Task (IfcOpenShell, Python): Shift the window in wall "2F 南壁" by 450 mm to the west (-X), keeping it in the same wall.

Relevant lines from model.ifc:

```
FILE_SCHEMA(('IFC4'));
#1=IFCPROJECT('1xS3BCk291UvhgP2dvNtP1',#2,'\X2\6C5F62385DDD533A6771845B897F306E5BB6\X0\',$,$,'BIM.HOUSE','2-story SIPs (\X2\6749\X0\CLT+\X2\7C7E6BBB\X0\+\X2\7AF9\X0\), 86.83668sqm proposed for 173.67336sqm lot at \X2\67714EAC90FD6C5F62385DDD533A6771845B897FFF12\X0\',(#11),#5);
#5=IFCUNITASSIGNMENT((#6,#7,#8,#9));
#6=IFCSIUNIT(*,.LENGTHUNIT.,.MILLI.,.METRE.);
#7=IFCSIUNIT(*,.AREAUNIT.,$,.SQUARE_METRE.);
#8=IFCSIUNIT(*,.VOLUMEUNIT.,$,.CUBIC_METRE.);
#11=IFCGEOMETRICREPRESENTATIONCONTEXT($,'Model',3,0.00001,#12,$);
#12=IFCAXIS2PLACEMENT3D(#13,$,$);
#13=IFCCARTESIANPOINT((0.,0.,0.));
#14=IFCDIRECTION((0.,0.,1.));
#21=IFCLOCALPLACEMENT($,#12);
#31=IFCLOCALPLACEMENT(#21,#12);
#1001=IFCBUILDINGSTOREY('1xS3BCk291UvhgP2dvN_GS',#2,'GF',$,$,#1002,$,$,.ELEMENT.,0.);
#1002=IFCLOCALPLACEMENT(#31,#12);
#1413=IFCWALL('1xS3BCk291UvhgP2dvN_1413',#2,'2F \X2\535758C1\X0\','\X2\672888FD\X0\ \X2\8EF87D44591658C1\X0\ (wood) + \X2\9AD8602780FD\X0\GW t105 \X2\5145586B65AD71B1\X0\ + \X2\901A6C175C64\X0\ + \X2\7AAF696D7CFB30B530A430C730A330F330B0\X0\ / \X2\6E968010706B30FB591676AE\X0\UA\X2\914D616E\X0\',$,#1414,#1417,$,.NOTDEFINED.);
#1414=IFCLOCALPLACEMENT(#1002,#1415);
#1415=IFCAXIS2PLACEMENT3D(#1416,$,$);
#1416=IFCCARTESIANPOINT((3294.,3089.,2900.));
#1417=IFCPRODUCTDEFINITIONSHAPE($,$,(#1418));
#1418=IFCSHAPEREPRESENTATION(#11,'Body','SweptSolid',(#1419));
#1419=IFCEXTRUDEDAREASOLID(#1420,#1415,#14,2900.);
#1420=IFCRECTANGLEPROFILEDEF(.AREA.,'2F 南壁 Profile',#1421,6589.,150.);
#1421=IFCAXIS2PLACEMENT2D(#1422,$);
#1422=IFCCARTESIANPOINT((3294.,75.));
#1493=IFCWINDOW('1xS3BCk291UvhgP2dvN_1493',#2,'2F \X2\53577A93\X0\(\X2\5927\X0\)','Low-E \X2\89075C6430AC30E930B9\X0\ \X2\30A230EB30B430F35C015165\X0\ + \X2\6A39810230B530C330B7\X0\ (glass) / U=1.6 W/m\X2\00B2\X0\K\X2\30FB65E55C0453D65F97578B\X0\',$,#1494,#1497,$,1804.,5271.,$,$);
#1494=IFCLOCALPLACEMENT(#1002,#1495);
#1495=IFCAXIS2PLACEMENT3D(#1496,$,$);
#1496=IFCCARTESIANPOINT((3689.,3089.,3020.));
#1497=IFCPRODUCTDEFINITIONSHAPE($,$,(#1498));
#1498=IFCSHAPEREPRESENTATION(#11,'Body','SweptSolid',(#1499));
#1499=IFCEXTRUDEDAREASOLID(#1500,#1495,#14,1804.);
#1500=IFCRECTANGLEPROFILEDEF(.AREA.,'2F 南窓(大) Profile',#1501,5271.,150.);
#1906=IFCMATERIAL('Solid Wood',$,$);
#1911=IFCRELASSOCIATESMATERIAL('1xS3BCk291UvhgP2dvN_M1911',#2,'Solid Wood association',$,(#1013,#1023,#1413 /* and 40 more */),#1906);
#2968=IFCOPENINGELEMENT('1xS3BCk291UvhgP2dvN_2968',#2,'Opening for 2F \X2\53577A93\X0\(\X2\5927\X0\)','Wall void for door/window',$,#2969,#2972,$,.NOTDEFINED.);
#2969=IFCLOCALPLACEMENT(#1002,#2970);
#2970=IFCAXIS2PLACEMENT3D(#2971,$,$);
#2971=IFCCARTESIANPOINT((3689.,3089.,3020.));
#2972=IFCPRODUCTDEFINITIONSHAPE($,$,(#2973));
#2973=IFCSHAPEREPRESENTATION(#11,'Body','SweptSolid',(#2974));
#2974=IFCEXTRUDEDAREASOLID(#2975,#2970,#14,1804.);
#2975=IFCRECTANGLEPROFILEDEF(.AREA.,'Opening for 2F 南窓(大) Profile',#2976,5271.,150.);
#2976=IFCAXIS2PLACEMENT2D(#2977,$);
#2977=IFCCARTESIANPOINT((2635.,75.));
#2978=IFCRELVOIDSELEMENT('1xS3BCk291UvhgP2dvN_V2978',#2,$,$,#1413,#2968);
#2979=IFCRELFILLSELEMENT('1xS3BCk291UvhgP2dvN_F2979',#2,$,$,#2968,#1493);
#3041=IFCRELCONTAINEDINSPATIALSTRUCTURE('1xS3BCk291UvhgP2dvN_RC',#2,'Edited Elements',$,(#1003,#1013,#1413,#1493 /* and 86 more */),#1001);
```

```python
import ifcopenshell
import ifcopenshell.api.geometry
import ifcopenshell.util.placement
import ifcopenshell.util.unit

model = ifcopenshell.open("model.ifc")
unit_scale = ifcopenshell.util.unit.calculate_unit_scale(model)

window = model.by_guid("1xS3BCk291UvhgP2dvN_1493")
opening = window.FillsVoids[0].RelatingOpeningElement
wall = opening.VoidsElements[0].RelatingBuildingElement

wall_matrix = ifcopenshell.util.placement.get_local_placement(wall.ObjectPlacement)
shift = wall_matrix[:3, 0] * -0.45 / unit_scale
before = ifcopenshell.util.placement.get_local_placement(window.ObjectPlacement)[:3, 3].copy()

# The window is not placed relative to its opening, so move both.
for product in (opening, window):
    matrix = ifcopenshell.util.placement.get_local_placement(product.ObjectPlacement)
    matrix[:3, 3] += shift
    ifcopenshell.api.geometry.edit_object_placement(model, product=product, matrix=matrix, is_si=False)

after = ifcopenshell.util.placement.get_local_placement(window.ObjectPlacement)[:3, 3]
print("window moved by", (after - before).round(3) + 0.0)

model.write("model_updated.ifc")
```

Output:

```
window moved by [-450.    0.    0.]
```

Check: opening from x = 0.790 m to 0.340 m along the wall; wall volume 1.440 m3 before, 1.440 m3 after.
